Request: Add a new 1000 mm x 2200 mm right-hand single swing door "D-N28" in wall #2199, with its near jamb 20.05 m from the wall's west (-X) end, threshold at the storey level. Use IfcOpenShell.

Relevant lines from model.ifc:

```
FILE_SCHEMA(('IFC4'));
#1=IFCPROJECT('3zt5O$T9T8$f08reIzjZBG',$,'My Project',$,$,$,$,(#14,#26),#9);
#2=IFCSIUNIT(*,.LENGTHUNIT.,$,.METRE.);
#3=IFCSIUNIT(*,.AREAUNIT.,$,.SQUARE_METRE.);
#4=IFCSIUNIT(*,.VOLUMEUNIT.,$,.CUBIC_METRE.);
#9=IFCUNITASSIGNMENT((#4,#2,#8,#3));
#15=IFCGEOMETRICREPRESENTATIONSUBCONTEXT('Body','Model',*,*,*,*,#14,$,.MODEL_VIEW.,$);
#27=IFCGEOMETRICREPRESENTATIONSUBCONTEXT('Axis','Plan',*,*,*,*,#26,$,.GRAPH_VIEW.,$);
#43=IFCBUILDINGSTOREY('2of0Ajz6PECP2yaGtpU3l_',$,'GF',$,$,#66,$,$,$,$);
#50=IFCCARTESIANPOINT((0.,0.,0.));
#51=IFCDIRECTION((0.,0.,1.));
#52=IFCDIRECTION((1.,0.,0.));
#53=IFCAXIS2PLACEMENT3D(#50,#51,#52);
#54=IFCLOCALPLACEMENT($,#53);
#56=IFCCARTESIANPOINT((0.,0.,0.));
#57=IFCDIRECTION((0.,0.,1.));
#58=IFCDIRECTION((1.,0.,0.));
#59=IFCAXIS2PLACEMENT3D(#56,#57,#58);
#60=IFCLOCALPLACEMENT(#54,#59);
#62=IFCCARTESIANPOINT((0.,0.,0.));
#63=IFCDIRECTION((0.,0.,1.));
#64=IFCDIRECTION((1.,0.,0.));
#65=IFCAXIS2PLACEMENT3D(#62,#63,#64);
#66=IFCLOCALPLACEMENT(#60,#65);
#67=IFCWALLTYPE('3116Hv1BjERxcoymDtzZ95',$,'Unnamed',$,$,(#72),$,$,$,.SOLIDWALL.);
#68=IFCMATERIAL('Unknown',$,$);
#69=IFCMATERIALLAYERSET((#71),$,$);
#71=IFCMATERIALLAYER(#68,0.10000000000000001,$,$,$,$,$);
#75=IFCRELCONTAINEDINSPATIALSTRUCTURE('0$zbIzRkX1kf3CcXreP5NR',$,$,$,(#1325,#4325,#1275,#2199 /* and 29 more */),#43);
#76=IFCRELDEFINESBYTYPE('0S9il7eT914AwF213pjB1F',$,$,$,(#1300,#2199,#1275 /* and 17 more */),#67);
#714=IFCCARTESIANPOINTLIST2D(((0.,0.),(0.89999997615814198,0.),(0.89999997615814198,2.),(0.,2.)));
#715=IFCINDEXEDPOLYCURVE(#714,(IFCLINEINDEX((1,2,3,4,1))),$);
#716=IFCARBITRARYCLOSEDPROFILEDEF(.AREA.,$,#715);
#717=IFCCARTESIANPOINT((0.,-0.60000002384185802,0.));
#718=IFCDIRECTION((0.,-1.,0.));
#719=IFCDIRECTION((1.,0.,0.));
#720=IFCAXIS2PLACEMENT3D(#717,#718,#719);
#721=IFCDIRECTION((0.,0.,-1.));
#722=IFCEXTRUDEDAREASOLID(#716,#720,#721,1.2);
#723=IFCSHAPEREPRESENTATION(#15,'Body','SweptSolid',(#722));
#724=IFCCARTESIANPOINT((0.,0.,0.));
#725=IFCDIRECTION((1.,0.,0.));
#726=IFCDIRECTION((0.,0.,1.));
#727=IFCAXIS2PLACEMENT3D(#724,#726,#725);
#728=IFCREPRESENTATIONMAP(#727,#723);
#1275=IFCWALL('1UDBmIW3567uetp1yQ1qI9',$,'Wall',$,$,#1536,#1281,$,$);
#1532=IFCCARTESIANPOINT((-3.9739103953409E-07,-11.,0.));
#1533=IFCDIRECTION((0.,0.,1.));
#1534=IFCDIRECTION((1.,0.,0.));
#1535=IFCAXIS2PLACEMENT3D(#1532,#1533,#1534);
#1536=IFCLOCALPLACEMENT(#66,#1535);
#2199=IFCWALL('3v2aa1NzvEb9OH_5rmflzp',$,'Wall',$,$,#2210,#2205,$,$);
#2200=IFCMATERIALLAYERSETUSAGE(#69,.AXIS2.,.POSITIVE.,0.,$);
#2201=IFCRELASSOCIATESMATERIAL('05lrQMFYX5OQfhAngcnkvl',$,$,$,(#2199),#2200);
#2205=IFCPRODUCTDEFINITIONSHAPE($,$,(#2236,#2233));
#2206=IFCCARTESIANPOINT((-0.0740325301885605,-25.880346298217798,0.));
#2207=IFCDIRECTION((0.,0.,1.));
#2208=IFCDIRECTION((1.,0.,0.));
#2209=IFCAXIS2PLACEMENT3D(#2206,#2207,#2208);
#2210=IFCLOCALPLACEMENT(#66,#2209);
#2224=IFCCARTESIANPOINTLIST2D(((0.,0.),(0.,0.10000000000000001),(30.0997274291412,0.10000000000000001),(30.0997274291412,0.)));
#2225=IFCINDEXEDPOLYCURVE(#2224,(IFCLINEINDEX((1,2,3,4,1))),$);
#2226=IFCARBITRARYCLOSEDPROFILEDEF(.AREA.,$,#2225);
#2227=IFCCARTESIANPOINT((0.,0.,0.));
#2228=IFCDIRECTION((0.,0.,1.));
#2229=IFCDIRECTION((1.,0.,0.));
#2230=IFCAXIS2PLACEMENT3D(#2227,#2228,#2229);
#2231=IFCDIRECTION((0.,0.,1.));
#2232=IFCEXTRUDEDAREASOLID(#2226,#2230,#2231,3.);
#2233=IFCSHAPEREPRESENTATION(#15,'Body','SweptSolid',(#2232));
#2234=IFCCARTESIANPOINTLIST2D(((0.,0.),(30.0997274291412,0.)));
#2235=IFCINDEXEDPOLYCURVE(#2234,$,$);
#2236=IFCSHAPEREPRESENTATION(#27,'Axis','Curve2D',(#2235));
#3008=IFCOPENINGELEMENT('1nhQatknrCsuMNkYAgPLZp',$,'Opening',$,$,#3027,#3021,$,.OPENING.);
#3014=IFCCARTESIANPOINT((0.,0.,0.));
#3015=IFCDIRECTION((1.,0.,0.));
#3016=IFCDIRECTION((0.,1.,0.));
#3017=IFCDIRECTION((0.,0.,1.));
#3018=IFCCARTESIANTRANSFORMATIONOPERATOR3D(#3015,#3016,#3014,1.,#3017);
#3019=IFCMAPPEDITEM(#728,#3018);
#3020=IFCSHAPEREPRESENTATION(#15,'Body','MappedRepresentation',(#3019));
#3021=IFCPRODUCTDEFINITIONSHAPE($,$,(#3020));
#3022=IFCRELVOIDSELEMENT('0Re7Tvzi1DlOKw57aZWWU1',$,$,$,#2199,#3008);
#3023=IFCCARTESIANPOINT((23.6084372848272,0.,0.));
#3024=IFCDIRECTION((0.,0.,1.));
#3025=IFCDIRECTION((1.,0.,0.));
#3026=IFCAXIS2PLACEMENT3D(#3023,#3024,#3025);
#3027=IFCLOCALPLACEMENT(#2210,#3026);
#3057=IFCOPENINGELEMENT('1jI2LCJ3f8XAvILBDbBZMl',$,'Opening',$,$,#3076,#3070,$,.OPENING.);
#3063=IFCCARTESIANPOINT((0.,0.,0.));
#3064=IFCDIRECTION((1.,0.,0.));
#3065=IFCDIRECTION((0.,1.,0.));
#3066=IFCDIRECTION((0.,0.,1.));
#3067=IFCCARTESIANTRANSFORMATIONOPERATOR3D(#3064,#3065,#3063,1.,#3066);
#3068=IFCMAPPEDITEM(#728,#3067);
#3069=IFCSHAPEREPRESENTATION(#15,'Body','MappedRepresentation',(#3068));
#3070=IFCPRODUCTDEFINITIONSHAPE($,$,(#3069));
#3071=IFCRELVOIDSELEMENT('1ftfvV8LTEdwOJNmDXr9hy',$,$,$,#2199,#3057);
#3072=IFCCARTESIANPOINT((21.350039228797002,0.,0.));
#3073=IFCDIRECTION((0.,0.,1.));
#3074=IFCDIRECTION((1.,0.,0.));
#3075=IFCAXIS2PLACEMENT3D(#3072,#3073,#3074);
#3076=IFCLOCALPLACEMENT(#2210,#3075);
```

```python
import numpy as np
import ifcopenshell
import ifcopenshell.api.feature
import ifcopenshell.api.geometry
import ifcopenshell.api.root
import ifcopenshell.api.spatial
import ifcopenshell.geom
import ifcopenshell.util.element
import ifcopenshell.util.placement
import ifcopenshell.util.representation
import ifcopenshell.util.shape
import ifcopenshell.util.unit

model = ifcopenshell.open("model.ifc")
unit_scale = ifcopenshell.util.unit.calculate_unit_scale(model)
settings = ifcopenshell.geom.settings()


def volume(element):
    """Net volume in cubic metres, openings subtracted."""
    shape = ifcopenshell.geom.create_shape(settings, element)
    return ifcopenshell.util.shape.get_volume(shape.geometry)


wall = model.by_guid("3v2aa1NzvEb9OH_5rmflzp")
storey = ifcopenshell.util.element.get_container(wall, ifc_class="IfcBuildingStorey")
context = ifcopenshell.util.representation.get_context(model, "Model", "Body", "MODEL_VIEW")
before = volume(wall)

width, height, from_end, sill = 1, 2.2, 20.05, 0.0  # metres

# The wall runs along its own X axis, and the end named is its -X end.
wall_shape = ifcopenshell.geom.create_shape(settings, wall)
x, y, z = ifcopenshell.util.shape.get_vertices(wall_shape.geometry).T
start = x.min() + from_end
face, thickness = float(y.min()), float(y.max() - y.min())
wall_matrix = ifcopenshell.util.placement.get_local_placement(wall.ObjectPlacement)
level = ifcopenshell.util.placement.get_local_placement(storey.ObjectPlacement)[2, 3]


def in_wall(x, y):
    """Placement at x, y metres in the wall's axes, at sill height."""
    matrix = wall_matrix.copy()
    matrix[:, 3] = wall_matrix @ np.array([x / unit_scale, y / unit_scale, 0.0, 1.0])
    matrix[2, 3] = level + sill / unit_scale
    return matrix


# Opening: a box that overshoots both wall faces by 50 mm.
opening = ifcopenshell.api.root.create_entity(model, ifc_class="IfcOpeningElement", predefined_type="OPENING")
box = ifcopenshell.api.geometry.add_wall_representation(
    model, context=context, length=width, height=height, thickness=thickness + 0.1
)
ifcopenshell.api.geometry.assign_representation(model, product=opening, representation=box)
ifcopenshell.api.geometry.edit_object_placement(model, product=opening, matrix=in_wall(start, face - 0.05), is_si=False)
ifcopenshell.api.feature.add_feature(model, feature=opening, element=wall)

door = ifcopenshell.api.root.create_entity(model, ifc_class="IfcDoor", name="D-N28", predefined_type="DOOR")
door.OverallWidth, door.OverallHeight = width / unit_scale, height / unit_scale
door.OperationType = "SINGLE_SWING_RIGHT"
body = ifcopenshell.api.geometry.add_door_representation(
    model,
    context=context,
    overall_width=door.OverallWidth,
    overall_height=door.OverallHeight,
    operation_type="SINGLE_SWING_RIGHT",
    lining_properties={"LiningDepth": thickness / unit_scale, "ThresholdDepth": thickness / unit_scale},
)
ifcopenshell.api.geometry.assign_representation(model, product=door, representation=body)
ifcopenshell.api.spatial.assign_container(model, products=[door], relating_structure=storey)
ifcopenshell.api.feature.add_filling(model, opening=opening, element=door)

# The lining spans the wall, so the door starts at the wall face.
ifcopenshell.api.geometry.edit_object_placement(model, product=door, matrix=in_wall(start, face), is_si=False)

after = volume(wall)

print(f"wall volume {before:.3f} -> {after:.3f} m3")

model.write("model_rev.ifc")
```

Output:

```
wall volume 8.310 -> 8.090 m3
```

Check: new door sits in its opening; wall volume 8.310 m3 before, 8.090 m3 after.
